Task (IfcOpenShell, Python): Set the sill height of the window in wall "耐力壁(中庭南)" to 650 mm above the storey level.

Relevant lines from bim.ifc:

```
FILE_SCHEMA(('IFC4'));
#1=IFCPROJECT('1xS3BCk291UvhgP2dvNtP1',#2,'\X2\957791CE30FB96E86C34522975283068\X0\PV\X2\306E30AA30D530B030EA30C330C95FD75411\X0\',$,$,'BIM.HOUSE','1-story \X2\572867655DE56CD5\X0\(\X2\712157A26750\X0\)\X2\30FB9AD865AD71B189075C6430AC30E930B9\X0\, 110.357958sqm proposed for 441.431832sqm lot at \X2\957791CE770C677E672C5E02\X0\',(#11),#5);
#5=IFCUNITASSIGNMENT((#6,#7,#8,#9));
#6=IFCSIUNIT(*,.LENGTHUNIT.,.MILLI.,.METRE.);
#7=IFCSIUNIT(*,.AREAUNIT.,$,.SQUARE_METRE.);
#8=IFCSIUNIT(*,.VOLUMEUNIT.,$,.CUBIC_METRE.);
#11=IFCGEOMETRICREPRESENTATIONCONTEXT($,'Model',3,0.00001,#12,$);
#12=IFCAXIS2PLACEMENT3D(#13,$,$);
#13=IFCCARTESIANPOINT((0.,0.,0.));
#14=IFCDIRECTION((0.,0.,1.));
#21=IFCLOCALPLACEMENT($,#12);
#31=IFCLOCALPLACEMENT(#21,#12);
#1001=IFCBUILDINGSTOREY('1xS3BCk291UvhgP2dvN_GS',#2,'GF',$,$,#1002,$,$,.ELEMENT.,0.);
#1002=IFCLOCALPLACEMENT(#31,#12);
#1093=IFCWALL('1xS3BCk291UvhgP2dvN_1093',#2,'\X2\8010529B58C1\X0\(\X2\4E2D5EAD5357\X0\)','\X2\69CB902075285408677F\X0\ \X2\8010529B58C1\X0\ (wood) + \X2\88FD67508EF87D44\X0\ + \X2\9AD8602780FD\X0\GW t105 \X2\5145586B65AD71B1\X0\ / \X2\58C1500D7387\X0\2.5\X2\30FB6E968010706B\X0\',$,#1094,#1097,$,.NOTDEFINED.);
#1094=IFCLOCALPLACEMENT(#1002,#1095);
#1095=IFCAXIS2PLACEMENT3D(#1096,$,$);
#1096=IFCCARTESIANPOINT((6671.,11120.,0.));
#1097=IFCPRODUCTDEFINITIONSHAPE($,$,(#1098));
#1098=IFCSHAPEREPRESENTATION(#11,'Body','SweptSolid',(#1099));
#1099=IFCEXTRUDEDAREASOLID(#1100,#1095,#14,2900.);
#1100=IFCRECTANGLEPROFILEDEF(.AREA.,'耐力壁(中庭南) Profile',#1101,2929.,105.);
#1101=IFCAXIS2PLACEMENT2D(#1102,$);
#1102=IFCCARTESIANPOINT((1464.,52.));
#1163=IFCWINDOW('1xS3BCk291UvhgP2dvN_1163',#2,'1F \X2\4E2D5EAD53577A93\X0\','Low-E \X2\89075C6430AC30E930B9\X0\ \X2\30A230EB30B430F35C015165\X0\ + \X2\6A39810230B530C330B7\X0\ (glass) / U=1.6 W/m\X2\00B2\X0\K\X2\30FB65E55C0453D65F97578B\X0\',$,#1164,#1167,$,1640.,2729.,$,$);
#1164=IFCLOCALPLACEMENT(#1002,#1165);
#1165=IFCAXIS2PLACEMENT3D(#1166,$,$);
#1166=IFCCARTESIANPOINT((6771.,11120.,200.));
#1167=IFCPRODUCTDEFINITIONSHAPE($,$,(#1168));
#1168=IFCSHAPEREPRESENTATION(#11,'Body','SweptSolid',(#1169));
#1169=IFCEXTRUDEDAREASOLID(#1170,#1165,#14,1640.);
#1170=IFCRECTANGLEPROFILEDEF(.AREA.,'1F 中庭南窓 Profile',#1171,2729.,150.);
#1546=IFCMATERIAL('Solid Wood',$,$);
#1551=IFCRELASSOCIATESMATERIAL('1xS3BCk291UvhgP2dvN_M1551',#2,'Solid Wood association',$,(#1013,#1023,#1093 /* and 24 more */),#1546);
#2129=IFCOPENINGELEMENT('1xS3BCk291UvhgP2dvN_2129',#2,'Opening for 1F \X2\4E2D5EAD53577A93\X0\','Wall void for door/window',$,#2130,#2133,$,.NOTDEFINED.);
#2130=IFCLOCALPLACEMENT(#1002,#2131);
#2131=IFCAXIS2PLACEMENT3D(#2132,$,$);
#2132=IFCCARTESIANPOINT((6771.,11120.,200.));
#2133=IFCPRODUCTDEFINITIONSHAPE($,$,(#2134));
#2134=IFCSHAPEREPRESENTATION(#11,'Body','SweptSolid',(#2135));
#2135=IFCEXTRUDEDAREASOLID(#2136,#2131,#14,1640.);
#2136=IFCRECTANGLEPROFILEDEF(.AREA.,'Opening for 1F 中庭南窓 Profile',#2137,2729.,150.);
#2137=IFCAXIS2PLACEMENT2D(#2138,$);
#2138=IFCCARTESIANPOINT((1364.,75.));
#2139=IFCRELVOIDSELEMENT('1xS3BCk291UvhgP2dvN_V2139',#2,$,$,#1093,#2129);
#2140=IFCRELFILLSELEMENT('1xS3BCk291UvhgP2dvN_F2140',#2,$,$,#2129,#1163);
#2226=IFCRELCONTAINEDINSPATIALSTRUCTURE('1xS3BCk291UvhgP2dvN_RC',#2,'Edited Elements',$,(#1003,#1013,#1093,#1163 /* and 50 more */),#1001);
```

```python
import numpy as np
import ifcopenshell
import ifcopenshell.api.geometry
import ifcopenshell.geom
import ifcopenshell.util.element
import ifcopenshell.util.placement
import ifcopenshell.util.shape
import ifcopenshell.util.unit

model = ifcopenshell.open("bim.ifc")
unit_scale = ifcopenshell.util.unit.calculate_unit_scale(model)

window = model.by_id(1163)
opening = window.FillsVoids[0].RelatingOpeningElement
storey = ifcopenshell.util.element.get_container(window, ifc_class="IfcBuildingStorey")
level = ifcopenshell.util.placement.get_local_placement(storey.ObjectPlacement)[2, 3]

# The opening's origin need not be at the sill, so measure its lowest point.
shape = ifcopenshell.geom.create_shape(ifcopenshell.geom.settings(), opening)
bottom = ifcopenshell.util.shape.get_shape_bottom_elevation(shape, shape.geometry) / unit_scale
dz = level + 0.65 / unit_scale - bottom

shift = np.array([0.0, 0.0, dz])
# The window is not placed relative to its opening, so move both.
for product in (opening, window):
    matrix = ifcopenshell.util.placement.get_local_placement(product.ObjectPlacement)
    matrix[:3, 3] += shift
    ifcopenshell.api.geometry.edit_object_placement(model, product=product, matrix=matrix, is_si=False)

print(f"moved by {dz * unit_scale:+.3f} m")

model.write("bim_updated.ifc")
```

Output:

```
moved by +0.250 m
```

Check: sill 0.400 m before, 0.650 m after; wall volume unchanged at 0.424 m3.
